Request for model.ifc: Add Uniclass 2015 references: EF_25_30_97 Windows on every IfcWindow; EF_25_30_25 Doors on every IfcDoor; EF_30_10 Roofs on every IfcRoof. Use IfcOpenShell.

First a look at what the model holds.

```python
import ifcopenshell

model = ifcopenshell.open("model.ifc")
print(model.schema)
print("classifications:", [c.Name for c in model.by_type("IfcClassification")])
for ifc_class in ("IfcDoor", "IfcRoof", "IfcStair", "IfcWall", "IfcWindow"):
    print(ifc_class, len(model.by_type(ifc_class)))
```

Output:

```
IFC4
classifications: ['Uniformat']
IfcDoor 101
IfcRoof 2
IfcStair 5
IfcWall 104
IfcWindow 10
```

```python
import ifcopenshell
import ifcopenshell.api.classification

model = ifcopenshell.open("model.ifc")

system = ifcopenshell.api.classification.add_classification(model, classification="Uniclass 2015")

codes = {
    "IfcWindow": ("EF_25_30_97", "Windows"),
    "IfcDoor": ("EF_25_30_25", "Doors"),
    "IfcRoof": ("EF_30_10", "Roofs"),
}
for ifc_class, (code, name) in codes.items():
    products = model.by_type(ifc_class)
    ifcopenshell.api.classification.add_reference(
        model, products=products, classification=system, identification=code, name=name
    )
    print(code, len(products))

model.write("model_updated.ifc")
```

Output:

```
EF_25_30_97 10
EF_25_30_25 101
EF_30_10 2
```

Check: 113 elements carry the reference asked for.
